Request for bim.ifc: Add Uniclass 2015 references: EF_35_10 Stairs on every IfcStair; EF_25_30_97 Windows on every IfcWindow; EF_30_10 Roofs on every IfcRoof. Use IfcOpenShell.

First a look at what the model holds.

```python
import ifcopenshell

model = ifcopenshell.open("bim.ifc")
print(model.schema)
print("classifications:", [c.Name for c in model.by_type("IfcClassification")])
for ifc_class in ("IfcDoor", "IfcRoof", "IfcStair", "IfcWall", "IfcWindow"):
    print(ifc_class, len(model.by_type(ifc_class)))
```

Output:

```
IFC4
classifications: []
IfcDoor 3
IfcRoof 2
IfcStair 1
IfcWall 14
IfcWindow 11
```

```python
import ifcopenshell
import ifcopenshell.api.classification

model = ifcopenshell.open("bim.ifc")

system = ifcopenshell.api.classification.add_classification(model, classification="Uniclass 2015")

codes = {
    "IfcStair": ("EF_35_10", "Stairs"),
    "IfcWindow": ("EF_25_30_97", "Windows"),
    "IfcRoof": ("EF_30_10", "Roofs"),
}
for ifc_class, (code, name) in codes.items():
    products = model.by_type(ifc_class)
    ifcopenshell.api.classification.add_reference(
        model, products=products, classification=system, identification=code, name=name
    )
    print(code, len(products))

model.write("bim-out.ifc")
```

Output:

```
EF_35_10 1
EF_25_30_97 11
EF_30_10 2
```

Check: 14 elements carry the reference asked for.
